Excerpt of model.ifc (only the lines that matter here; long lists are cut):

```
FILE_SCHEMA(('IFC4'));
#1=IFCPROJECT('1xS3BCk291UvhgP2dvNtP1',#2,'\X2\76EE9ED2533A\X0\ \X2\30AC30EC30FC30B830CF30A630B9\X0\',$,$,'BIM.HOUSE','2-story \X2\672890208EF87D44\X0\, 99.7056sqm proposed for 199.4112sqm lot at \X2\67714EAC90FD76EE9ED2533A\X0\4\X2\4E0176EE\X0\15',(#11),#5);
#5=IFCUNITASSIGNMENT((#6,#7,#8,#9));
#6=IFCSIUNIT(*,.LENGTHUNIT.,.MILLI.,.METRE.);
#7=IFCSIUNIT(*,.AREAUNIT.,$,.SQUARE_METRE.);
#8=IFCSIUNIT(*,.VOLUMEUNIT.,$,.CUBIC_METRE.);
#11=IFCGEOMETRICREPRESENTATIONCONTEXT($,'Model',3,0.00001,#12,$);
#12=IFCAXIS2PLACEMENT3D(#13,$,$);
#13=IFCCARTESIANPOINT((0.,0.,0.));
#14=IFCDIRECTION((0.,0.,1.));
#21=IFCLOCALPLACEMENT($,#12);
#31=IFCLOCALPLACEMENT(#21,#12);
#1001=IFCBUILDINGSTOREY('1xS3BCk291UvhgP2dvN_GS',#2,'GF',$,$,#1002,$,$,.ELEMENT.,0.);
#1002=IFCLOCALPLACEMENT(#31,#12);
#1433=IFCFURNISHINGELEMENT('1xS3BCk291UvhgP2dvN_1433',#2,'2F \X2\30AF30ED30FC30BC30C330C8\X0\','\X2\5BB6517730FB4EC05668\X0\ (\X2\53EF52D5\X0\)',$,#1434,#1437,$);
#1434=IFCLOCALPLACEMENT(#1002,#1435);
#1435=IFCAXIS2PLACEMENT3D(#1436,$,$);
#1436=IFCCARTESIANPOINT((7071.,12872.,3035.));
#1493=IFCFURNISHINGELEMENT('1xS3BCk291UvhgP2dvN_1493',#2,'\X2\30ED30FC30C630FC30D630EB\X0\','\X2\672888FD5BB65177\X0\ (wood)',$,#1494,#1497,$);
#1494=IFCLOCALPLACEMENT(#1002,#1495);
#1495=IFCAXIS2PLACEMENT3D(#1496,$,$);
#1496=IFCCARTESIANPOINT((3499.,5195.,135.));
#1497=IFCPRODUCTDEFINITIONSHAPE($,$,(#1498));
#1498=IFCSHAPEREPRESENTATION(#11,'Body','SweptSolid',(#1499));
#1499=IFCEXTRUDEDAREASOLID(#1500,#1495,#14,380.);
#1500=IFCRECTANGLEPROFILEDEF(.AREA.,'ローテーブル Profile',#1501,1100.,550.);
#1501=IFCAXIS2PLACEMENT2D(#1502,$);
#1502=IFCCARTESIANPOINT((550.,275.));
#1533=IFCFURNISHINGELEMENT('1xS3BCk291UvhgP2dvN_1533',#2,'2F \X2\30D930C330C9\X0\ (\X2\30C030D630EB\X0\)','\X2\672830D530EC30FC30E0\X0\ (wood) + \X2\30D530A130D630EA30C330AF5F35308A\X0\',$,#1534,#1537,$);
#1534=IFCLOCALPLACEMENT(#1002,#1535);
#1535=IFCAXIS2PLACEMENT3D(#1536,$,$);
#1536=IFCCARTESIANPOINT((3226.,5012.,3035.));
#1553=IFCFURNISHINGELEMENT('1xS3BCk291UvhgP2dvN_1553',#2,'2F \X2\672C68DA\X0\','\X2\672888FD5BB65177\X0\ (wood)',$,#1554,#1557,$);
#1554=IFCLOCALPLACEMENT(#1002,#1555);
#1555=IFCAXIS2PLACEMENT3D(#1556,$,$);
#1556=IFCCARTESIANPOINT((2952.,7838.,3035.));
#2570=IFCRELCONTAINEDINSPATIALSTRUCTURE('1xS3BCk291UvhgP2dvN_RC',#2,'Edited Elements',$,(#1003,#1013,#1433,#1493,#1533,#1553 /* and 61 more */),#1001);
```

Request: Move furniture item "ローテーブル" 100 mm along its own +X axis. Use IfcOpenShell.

```python
import ifcopenshell
import ifcopenshell.api.geometry
import ifcopenshell.util.placement
import ifcopenshell.util.unit

model = ifcopenshell.open("model.ifc")
unit_scale = ifcopenshell.util.unit.calculate_unit_scale(model)

item = model.by_guid("1xS3BCk291UvhgP2dvN_1493")
matrix = ifcopenshell.util.placement.get_local_placement(item.ObjectPlacement)
matrix[:3, 3] += matrix[:3, 0] * 0.1 / unit_scale
ifcopenshell.api.geometry.edit_object_placement(model, product=item, matrix=matrix, is_si=False)

print(ifcopenshell.util.placement.get_local_placement(item.ObjectPlacement).round(3) + 0.0)

model.write("model_edited.ifc")
```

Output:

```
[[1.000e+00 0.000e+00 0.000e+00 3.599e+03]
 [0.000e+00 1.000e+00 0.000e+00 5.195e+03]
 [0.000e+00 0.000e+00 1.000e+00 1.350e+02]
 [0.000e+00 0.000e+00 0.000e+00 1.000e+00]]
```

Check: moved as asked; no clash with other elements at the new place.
